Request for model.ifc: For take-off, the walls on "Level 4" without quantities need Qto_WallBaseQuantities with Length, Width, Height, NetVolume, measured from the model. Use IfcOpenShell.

First a look at what the model holds.

```python
import ifcopenshell
import ifcopenshell.util.element
import ifcopenshell.util.unit

model = ifcopenshell.open("model.ifc")
print(model.schema)
for unit_type in ("LENGTHUNIT", "AREAUNIT", "VOLUMEUNIT"):
    print(unit_type, ifcopenshell.util.unit.calculate_unit_scale(model, unit_type))
storey = next(s for s in model.by_type("IfcBuildingStorey") if s.Name == "Level 4")
walls = [e for e in ifcopenshell.util.element.get_decomposition(storey) if e.is_a("IfcWall")]
for e in sorted(walls, key=lambda e: e.id()):
    print(e.id(), e.is_a(), e.Name, list(ifcopenshell.util.element.get_psets(e, qtos_only=True)), sep=" | ")
```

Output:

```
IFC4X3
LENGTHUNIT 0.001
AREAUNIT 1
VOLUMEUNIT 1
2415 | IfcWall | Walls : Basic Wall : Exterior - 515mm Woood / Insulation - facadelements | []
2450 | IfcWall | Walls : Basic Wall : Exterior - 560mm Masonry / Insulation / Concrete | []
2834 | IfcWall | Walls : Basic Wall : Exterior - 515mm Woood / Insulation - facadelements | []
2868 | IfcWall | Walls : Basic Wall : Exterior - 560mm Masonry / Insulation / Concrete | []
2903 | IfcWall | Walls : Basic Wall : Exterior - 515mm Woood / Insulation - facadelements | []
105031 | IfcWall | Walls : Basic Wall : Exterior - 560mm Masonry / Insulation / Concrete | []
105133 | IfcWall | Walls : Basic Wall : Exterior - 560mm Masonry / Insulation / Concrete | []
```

```python
import ifcopenshell
import ifcopenshell.api.pset
import ifcopenshell.geom
import ifcopenshell.util.element
import ifcopenshell.util.shape
import ifcopenshell.util.unit

model = ifcopenshell.open("model.ifc")
unit_scale = ifcopenshell.util.unit.calculate_unit_scale(model)
volume_scale = ifcopenshell.util.unit.calculate_unit_scale(model, "VOLUMEUNIT")
settings = ifcopenshell.geom.settings()

storey = next(s for s in model.by_type("IfcBuildingStorey") if s.Name == "Level 4")
walls = [e for e in ifcopenshell.util.element.get_decomposition(storey) if e.is_a("IfcWall")]

for e in sorted(walls, key=lambda e: e.id()):
    if ifcopenshell.util.element.get_psets(e, qtos_only=True, should_inherit=False):
        continue
    # Geometry comes back in metres, in the element's own axes.
    shape = ifcopenshell.geom.create_shape(settings, e)
    values = {
        "Length": ifcopenshell.util.shape.get_x(shape.geometry) / unit_scale,
        "Width": ifcopenshell.util.shape.get_y(shape.geometry) / unit_scale,
        "Height": ifcopenshell.util.shape.get_z(shape.geometry) / unit_scale,
        "NetVolume": ifcopenshell.util.shape.get_volume(shape.geometry) / volume_scale,
    }
    qto = ifcopenshell.api.pset.add_qto(model, product=e, name="Qto_WallBaseQuantities")
    ifcopenshell.api.pset.edit_qto(model, qto=qto, properties=values)
    print(e.id(), {k: round(v, 3) for k, v in values.items()})

model.write("model_v2.ifc")
```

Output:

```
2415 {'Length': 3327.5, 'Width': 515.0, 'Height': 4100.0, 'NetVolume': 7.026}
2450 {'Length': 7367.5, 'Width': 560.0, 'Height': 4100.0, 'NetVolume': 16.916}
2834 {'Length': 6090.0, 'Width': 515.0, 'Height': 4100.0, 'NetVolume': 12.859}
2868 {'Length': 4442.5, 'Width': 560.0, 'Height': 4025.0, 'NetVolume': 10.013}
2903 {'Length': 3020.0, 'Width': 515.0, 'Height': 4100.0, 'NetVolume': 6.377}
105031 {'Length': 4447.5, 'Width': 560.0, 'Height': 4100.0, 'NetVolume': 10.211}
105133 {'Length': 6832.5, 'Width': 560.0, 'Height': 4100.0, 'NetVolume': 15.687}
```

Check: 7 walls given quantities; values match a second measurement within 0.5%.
